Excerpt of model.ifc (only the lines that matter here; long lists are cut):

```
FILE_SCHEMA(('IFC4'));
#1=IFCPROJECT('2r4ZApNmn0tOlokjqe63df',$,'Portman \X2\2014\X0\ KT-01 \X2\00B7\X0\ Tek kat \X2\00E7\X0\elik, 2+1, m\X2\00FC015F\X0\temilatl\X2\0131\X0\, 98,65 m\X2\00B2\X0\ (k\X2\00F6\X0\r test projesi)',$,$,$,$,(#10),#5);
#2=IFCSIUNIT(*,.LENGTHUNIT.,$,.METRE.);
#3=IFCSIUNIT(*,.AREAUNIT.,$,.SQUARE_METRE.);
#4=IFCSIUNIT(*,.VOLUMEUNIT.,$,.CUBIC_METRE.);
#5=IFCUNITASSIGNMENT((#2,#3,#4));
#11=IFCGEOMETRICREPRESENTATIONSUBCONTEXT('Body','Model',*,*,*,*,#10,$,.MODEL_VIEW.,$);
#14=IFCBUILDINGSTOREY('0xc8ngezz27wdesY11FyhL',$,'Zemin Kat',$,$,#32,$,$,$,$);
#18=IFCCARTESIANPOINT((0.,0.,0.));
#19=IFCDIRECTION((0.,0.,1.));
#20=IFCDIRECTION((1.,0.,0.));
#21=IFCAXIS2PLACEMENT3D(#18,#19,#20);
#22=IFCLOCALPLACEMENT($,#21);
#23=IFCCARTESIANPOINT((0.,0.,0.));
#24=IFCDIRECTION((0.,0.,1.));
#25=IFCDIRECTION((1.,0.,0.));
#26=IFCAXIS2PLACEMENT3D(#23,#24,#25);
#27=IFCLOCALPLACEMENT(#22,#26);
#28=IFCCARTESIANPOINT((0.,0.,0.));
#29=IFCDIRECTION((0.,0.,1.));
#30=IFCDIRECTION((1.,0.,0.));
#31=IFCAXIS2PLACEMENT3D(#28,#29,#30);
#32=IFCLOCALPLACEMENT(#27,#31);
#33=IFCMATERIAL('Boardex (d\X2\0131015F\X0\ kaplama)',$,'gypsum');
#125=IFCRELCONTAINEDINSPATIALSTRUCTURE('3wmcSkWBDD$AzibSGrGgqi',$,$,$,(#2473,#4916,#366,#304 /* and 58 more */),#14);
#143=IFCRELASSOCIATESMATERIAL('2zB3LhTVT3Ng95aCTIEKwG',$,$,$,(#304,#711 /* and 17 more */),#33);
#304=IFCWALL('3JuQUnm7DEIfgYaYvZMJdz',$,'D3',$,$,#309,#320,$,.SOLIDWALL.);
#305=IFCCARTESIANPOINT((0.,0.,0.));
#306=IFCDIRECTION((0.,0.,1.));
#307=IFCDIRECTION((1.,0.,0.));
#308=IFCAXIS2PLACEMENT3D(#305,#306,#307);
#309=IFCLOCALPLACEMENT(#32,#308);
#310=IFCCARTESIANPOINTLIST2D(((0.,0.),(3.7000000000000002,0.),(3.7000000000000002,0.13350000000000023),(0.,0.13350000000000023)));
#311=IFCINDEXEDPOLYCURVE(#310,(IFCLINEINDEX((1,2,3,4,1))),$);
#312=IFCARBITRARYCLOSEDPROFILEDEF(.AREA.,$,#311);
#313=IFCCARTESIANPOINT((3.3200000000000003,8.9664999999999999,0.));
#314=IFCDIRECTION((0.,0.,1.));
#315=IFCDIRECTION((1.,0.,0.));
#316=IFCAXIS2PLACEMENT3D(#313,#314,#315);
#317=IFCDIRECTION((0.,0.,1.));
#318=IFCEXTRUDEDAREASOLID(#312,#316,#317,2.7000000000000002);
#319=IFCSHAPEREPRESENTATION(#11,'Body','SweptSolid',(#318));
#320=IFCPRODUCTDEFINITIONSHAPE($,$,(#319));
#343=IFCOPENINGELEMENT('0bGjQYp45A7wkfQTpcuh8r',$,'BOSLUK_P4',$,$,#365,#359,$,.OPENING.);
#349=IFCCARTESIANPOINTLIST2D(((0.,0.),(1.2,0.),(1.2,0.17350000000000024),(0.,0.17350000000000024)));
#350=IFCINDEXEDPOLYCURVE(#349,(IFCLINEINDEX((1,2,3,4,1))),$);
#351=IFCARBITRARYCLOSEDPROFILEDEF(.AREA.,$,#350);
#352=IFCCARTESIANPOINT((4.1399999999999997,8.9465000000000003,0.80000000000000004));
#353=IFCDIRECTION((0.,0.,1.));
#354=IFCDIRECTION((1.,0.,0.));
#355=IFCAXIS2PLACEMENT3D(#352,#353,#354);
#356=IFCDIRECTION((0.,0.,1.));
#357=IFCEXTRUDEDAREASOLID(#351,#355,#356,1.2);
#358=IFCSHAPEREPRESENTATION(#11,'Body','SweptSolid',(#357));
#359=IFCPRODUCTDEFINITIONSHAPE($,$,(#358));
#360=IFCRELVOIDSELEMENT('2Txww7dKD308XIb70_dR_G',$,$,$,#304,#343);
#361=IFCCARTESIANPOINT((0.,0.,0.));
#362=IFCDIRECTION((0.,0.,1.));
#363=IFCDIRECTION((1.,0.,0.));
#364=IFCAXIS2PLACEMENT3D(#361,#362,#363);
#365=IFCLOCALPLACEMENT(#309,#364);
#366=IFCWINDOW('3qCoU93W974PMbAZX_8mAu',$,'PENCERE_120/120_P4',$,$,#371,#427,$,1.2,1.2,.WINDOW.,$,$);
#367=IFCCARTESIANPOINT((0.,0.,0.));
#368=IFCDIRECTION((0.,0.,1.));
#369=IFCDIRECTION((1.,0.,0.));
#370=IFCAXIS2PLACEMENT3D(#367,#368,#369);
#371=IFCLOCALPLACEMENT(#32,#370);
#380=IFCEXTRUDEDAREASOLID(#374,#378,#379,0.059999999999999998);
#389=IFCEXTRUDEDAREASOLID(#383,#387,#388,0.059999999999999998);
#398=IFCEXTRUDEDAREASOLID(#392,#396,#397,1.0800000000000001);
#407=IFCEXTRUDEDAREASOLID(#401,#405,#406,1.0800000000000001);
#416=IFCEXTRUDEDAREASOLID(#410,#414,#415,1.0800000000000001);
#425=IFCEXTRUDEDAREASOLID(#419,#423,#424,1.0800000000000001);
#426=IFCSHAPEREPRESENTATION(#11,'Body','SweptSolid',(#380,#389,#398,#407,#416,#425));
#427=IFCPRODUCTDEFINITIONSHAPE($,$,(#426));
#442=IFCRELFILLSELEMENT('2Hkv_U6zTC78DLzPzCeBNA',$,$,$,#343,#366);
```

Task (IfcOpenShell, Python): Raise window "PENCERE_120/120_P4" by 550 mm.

```python
import numpy as np
import ifcopenshell
import ifcopenshell.api.geometry
import ifcopenshell.util.placement
import ifcopenshell.util.unit

model = ifcopenshell.open("model.ifc")
unit_scale = ifcopenshell.util.unit.calculate_unit_scale(model)

window = model.by_guid("3qCoU93W974PMbAZX_8mAu")
opening = window.FillsVoids[0].RelatingOpeningElement
dz = 0.55

shift = np.array([0.0, 0.0, dz])
# The window is not placed relative to its opening, so move both.
for product in (opening, window):
    matrix = ifcopenshell.util.placement.get_local_placement(product.ObjectPlacement)
    matrix[:3, 3] += shift
    ifcopenshell.api.geometry.edit_object_placement(model, product=product, matrix=matrix, is_si=False)

print(f"moved by {dz * unit_scale:+.3f} m")

model.write("model_rev.ifc")
```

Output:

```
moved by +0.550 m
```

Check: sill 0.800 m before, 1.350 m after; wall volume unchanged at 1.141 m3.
